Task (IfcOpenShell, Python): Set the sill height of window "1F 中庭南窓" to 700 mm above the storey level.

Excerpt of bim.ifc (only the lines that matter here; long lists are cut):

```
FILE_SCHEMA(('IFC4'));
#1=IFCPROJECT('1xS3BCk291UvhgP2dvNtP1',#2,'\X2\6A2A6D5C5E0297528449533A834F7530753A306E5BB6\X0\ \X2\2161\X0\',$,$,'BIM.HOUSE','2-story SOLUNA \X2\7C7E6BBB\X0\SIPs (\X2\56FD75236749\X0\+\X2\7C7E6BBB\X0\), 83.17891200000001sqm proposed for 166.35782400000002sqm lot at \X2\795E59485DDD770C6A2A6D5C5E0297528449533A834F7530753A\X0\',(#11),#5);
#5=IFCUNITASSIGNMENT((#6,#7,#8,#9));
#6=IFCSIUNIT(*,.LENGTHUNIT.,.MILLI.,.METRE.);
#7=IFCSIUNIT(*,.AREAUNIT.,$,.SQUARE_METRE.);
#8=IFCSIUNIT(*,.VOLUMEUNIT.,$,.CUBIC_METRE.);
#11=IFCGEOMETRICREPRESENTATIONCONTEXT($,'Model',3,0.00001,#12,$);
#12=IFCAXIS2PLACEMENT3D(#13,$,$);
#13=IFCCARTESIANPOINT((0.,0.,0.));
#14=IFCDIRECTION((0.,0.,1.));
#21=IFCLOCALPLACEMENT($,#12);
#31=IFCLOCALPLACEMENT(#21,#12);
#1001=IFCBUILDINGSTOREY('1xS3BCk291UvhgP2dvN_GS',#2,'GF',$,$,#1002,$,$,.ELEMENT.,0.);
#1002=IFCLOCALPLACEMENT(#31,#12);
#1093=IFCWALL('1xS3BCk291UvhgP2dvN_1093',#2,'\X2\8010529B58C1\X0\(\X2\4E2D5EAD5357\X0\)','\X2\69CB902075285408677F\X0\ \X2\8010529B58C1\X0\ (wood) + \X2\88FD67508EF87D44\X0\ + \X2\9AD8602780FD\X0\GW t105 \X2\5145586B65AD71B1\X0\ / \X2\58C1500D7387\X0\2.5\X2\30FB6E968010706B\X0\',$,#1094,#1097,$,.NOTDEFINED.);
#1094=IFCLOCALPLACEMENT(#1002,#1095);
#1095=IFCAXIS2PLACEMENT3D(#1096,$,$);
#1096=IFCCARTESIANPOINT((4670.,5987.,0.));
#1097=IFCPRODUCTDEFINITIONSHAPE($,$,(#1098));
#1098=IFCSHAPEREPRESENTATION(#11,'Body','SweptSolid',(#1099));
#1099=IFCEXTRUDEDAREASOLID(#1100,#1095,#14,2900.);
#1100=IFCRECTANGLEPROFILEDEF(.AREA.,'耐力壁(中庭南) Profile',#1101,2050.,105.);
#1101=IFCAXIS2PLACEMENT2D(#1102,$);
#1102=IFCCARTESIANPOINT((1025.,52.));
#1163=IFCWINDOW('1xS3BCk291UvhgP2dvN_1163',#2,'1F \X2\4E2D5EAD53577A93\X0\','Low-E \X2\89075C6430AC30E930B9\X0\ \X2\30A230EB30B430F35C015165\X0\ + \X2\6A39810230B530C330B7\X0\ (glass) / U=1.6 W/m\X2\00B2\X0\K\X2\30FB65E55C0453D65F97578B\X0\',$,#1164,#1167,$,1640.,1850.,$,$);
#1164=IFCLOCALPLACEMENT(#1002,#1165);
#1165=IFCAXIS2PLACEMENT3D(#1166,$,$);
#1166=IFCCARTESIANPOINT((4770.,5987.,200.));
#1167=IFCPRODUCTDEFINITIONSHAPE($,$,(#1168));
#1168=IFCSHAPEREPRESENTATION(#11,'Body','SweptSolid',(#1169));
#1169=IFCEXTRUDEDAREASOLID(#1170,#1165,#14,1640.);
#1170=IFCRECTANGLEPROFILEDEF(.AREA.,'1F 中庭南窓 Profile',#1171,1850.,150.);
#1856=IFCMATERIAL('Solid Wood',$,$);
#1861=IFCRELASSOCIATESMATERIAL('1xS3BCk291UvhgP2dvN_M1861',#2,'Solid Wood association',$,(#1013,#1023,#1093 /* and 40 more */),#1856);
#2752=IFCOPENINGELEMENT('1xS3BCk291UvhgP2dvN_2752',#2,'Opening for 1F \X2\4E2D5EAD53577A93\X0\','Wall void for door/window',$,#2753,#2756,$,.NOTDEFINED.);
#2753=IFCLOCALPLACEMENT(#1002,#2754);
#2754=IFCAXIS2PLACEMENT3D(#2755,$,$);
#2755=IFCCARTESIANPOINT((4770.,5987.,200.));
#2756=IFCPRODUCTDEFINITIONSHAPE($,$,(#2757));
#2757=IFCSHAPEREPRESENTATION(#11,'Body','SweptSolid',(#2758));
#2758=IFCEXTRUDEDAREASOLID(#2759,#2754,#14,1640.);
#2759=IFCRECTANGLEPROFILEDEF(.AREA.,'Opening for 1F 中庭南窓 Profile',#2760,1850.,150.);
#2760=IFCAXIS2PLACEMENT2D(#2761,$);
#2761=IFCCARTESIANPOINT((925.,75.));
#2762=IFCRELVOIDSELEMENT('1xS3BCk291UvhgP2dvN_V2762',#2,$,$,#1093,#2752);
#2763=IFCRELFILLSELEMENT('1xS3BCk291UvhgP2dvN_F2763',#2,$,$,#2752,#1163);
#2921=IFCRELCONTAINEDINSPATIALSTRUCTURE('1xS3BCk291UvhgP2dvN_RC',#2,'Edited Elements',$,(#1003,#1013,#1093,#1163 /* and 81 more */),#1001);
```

```python
import numpy as np
import ifcopenshell
import ifcopenshell.api.geometry
import ifcopenshell.geom
import ifcopenshell.util.element
import ifcopenshell.util.placement
import ifcopenshell.util.shape
import ifcopenshell.util.unit

model = ifcopenshell.open("bim.ifc")
unit_scale = ifcopenshell.util.unit.calculate_unit_scale(model)

window = model.by_guid("1xS3BCk291UvhgP2dvN_1163")
opening = window.FillsVoids[0].RelatingOpeningElement
storey = ifcopenshell.util.element.get_container(window, ifc_class="IfcBuildingStorey")
level = ifcopenshell.util.placement.get_local_placement(storey.ObjectPlacement)[2, 3]

# The opening's origin need not be at the sill, so measure its lowest point.
shape = ifcopenshell.geom.create_shape(ifcopenshell.geom.settings(), opening)
bottom = ifcopenshell.util.shape.get_shape_bottom_elevation(shape, shape.geometry) / unit_scale
dz = level + 700.0 - bottom

shift = np.array([0.0, 0.0, dz])
# The window is not placed relative to its opening, so move both.
for product in (opening, window):
    matrix = ifcopenshell.util.placement.get_local_placement(product.ObjectPlacement)
    matrix[:3, 3] += shift
    ifcopenshell.api.geometry.edit_object_placement(model, product=product, matrix=matrix, is_si=False)

print(f"moved by {dz * unit_scale:+.3f} m")

model.write("bim_rev.ifc")
```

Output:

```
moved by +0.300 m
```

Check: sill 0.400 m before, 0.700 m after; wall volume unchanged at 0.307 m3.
